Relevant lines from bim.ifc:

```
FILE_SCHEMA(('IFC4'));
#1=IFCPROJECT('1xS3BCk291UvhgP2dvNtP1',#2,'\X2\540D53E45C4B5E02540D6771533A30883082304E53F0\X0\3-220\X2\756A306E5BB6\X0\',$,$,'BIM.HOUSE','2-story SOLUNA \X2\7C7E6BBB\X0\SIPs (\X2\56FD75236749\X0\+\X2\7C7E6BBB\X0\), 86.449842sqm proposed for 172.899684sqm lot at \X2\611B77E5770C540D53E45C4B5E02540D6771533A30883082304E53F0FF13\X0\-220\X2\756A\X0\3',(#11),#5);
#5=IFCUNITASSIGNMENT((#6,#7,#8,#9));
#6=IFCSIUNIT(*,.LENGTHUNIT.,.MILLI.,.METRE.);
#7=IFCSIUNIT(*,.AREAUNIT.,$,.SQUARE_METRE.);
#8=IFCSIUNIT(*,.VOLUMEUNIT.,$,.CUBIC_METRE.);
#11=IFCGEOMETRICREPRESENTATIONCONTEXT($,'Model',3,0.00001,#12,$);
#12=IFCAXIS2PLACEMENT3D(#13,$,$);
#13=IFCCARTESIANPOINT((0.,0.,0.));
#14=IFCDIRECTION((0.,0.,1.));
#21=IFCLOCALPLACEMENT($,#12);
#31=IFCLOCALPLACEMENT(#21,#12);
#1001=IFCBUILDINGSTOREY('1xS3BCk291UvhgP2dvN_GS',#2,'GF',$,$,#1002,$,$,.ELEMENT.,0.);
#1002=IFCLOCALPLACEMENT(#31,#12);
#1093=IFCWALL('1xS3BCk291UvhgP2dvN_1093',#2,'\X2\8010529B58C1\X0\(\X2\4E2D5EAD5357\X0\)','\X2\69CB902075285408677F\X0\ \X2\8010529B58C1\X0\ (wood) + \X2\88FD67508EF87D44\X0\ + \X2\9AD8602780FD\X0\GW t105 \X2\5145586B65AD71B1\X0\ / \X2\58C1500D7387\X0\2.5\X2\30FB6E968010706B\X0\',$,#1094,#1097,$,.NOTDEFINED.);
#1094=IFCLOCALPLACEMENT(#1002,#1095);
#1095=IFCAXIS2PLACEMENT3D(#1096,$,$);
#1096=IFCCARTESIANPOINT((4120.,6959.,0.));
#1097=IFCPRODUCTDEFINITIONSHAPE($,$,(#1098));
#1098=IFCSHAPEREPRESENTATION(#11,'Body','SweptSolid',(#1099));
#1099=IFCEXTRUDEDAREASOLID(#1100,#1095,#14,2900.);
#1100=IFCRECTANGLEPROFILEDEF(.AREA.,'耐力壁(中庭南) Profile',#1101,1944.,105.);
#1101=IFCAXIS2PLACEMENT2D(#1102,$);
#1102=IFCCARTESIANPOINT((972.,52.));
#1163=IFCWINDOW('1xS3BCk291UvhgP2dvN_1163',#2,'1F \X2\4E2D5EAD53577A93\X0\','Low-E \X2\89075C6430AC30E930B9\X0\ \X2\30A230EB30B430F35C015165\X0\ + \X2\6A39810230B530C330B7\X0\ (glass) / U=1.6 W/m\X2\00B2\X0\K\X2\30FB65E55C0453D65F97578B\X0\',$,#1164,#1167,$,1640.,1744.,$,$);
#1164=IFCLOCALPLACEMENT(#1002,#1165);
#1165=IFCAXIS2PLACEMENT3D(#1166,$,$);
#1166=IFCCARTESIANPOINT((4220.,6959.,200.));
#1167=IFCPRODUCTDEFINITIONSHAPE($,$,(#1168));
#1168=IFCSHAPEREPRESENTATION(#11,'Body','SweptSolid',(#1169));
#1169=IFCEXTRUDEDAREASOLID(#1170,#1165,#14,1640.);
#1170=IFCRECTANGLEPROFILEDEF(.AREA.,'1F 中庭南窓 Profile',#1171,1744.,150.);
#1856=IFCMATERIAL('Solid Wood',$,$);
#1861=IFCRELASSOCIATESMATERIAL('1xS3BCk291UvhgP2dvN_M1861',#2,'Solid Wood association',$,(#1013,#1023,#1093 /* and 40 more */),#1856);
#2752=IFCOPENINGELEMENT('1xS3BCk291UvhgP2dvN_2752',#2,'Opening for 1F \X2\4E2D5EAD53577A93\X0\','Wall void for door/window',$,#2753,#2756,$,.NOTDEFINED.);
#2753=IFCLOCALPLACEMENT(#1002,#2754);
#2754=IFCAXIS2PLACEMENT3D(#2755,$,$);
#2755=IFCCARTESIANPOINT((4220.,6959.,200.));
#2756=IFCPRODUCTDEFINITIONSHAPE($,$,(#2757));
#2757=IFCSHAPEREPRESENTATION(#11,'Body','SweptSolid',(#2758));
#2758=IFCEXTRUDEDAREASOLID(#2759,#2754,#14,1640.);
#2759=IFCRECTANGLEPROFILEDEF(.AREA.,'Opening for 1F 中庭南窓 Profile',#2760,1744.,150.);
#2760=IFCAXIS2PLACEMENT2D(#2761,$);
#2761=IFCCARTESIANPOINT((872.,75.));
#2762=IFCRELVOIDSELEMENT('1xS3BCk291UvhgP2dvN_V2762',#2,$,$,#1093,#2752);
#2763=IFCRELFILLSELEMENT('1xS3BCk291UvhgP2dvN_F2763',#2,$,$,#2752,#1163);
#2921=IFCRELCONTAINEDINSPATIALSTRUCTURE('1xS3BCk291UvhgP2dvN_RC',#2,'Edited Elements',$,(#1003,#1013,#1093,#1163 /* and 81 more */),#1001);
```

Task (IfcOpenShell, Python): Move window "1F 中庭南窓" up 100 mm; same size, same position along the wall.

```python
import numpy as np
import ifcopenshell
import ifcopenshell.api.geometry
import ifcopenshell.util.placement
import ifcopenshell.util.unit

model = ifcopenshell.open("bim.ifc")
unit_scale = ifcopenshell.util.unit.calculate_unit_scale(model)

window = model.by_id(1163)
opening = window.FillsVoids[0].RelatingOpeningElement
dz = 0.1 / unit_scale

shift = np.array([0.0, 0.0, dz])
# The window is not placed relative to its opening, so move both.
for product in (opening, window):
    matrix = ifcopenshell.util.placement.get_local_placement(product.ObjectPlacement)
    matrix[:3, 3] += shift
    ifcopenshell.api.geometry.edit_object_placement(model, product=product, matrix=matrix, is_si=False)

print(f"moved by {dz * unit_scale:+.3f} m")

model.write("bim_updated.ifc")
```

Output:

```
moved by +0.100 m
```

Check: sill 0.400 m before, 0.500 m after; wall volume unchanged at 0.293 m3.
